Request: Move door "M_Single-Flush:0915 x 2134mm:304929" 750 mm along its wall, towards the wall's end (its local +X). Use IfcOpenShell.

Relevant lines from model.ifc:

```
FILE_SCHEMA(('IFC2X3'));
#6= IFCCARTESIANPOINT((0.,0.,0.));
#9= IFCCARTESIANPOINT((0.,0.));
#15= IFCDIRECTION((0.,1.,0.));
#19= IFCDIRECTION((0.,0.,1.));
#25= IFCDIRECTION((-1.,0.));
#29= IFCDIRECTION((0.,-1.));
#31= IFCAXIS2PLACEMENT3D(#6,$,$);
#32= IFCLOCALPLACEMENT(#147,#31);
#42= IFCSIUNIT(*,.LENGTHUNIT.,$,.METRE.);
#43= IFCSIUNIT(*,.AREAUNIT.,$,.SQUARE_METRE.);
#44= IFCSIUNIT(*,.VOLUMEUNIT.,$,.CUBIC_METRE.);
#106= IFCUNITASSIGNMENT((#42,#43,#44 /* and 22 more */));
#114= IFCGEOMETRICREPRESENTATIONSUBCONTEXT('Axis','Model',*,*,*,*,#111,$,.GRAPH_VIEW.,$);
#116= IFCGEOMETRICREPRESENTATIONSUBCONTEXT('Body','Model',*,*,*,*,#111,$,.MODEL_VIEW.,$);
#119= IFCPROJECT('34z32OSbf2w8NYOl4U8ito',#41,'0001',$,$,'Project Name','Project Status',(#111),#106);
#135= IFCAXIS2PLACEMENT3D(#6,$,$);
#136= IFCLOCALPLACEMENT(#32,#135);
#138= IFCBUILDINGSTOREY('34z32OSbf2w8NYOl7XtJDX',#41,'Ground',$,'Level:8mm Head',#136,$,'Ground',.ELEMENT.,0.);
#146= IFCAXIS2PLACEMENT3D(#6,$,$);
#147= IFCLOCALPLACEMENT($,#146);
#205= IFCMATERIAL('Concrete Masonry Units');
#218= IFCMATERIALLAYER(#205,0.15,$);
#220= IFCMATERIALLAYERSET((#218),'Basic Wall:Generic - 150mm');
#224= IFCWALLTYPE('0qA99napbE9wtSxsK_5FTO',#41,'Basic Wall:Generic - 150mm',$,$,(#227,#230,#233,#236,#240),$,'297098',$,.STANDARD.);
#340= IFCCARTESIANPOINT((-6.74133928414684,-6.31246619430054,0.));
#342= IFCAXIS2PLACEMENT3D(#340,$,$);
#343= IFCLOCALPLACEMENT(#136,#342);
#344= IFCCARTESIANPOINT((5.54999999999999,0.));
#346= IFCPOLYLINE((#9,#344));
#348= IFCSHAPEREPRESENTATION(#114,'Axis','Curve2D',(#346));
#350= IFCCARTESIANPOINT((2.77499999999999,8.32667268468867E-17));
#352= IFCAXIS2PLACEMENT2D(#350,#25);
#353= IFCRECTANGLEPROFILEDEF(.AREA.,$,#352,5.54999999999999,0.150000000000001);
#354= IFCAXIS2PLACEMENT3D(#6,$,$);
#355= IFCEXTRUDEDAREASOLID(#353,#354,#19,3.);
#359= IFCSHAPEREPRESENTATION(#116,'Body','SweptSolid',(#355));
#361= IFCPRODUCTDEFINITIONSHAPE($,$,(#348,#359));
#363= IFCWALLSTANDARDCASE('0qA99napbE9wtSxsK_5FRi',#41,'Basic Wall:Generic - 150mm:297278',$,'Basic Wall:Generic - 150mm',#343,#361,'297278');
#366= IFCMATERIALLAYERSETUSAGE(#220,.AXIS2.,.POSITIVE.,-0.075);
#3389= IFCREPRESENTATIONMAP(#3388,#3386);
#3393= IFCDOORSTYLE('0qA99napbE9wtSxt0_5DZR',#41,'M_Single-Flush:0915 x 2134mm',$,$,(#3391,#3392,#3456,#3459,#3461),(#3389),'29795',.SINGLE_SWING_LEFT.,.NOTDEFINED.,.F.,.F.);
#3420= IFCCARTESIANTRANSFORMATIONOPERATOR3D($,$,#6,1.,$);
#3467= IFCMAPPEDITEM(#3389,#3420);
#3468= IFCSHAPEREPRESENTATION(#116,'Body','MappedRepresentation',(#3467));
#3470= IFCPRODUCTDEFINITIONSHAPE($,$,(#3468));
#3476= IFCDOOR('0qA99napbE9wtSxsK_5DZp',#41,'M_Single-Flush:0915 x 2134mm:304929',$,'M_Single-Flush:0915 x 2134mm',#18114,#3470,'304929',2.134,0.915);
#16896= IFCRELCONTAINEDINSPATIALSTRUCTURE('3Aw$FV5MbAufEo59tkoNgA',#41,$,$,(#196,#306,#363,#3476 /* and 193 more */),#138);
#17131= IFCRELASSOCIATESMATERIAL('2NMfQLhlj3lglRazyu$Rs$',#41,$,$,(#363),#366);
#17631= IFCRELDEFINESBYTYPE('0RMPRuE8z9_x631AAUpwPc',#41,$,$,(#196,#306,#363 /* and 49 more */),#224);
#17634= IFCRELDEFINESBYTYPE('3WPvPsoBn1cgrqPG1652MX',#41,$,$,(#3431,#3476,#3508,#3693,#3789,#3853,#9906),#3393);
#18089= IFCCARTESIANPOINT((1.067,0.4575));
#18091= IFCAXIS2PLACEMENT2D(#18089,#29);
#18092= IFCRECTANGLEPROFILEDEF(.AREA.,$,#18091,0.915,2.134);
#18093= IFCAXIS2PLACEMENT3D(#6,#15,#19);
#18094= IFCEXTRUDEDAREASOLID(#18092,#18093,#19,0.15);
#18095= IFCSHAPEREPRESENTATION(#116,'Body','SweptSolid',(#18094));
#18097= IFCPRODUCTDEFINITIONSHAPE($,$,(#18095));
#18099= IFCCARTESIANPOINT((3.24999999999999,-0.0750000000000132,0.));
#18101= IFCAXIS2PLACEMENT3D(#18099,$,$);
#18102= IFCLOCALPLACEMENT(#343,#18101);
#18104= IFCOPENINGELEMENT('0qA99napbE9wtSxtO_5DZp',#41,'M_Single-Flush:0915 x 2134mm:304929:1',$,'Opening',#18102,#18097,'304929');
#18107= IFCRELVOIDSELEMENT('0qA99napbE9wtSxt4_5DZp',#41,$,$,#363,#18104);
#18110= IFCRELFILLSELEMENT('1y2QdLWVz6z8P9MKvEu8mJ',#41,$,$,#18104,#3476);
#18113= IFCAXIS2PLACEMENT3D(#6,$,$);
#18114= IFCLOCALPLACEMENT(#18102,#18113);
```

```python
import ifcopenshell
import ifcopenshell.api.geometry
import ifcopenshell.util.placement
import ifcopenshell.util.unit

model = ifcopenshell.open("model.ifc")
unit_scale = ifcopenshell.util.unit.calculate_unit_scale(model)

door = model.by_guid("0qA99napbE9wtSxsK_5DZp")
opening = door.FillsVoids[0].RelatingOpeningElement
wall = opening.VoidsElements[0].RelatingBuildingElement

wall_matrix = ifcopenshell.util.placement.get_local_placement(wall.ObjectPlacement)
shift = wall_matrix[:3, 0] * 0.75 / unit_scale
before = ifcopenshell.util.placement.get_local_placement(door.ObjectPlacement)[:3, 3].copy()

# The door is placed relative to its opening, so it follows when the opening moves.
matrix = ifcopenshell.util.placement.get_local_placement(opening.ObjectPlacement)
matrix[:3, 3] += shift
ifcopenshell.api.geometry.edit_object_placement(
    model, product=opening, matrix=matrix, is_si=False, should_transform_children=True
)

after = ifcopenshell.util.placement.get_local_placement(door.ObjectPlacement)[:3, 3]
print("door moved by", (after - before).round(3) + 0.0)

model.write("model-out.ifc")
```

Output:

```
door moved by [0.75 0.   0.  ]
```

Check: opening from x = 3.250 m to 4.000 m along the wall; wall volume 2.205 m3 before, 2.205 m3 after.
